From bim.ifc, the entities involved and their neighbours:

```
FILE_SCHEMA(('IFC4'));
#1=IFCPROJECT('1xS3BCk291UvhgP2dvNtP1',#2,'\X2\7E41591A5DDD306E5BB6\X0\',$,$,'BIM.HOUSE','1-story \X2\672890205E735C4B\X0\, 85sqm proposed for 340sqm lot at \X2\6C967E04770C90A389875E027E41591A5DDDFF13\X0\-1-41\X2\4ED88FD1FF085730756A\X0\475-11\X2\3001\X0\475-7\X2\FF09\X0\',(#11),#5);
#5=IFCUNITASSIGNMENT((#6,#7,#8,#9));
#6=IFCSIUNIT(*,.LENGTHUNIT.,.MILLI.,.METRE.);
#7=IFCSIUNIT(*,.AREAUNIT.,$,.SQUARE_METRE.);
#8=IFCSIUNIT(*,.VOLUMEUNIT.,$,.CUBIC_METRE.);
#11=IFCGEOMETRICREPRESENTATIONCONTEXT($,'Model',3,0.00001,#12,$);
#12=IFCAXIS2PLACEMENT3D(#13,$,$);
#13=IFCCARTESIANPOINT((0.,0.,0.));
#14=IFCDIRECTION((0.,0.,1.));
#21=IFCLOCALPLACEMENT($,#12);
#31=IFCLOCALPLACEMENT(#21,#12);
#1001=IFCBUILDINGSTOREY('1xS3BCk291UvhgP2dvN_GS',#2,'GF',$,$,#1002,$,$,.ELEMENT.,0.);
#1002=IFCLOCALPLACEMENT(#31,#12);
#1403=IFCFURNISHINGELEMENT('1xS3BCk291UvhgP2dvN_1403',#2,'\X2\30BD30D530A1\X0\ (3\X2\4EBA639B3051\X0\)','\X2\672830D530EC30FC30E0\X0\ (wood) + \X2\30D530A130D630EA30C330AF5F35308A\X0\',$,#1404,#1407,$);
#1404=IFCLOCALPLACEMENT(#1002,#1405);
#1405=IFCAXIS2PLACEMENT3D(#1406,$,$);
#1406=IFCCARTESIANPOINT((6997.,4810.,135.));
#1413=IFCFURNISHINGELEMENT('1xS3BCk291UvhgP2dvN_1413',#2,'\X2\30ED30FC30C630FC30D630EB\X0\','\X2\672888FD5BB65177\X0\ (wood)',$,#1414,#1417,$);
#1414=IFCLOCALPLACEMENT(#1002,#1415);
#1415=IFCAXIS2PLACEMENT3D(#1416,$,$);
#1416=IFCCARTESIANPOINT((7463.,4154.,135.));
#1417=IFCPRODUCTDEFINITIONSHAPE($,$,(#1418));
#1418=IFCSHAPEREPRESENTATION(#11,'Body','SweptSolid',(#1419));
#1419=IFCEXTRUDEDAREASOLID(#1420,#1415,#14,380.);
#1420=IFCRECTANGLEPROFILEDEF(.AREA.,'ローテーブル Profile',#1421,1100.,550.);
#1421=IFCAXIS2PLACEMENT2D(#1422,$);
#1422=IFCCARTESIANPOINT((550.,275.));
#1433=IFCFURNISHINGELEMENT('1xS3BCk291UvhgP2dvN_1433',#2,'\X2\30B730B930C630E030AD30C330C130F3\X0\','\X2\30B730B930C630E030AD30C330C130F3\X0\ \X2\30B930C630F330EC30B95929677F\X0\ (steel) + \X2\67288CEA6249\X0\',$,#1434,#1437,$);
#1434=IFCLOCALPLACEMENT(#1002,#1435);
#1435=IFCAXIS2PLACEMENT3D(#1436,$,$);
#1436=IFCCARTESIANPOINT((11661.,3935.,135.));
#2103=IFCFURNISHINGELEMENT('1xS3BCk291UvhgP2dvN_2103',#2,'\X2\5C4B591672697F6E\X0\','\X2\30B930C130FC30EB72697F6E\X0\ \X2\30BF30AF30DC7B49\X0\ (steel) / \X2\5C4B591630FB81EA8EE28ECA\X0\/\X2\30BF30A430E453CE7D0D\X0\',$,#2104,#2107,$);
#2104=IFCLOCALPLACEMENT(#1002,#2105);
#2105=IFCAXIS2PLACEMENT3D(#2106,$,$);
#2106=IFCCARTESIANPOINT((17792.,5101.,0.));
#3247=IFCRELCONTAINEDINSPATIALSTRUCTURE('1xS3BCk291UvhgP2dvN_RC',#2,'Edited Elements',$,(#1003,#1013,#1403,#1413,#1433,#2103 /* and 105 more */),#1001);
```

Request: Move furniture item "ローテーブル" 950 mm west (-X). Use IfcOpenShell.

```python
import ifcopenshell
import ifcopenshell.api.geometry
import ifcopenshell.util.placement
import ifcopenshell.util.unit

model = ifcopenshell.open("bim.ifc")
unit_scale = ifcopenshell.util.unit.calculate_unit_scale(model)

item = model.by_id(1413)
matrix = ifcopenshell.util.placement.get_local_placement(item.ObjectPlacement)
matrix[0, 3] -= 0.95 / unit_scale
ifcopenshell.api.geometry.edit_object_placement(model, product=item, matrix=matrix, is_si=False)

print(ifcopenshell.util.placement.get_local_placement(item.ObjectPlacement).round(3) + 0.0)

model.write("bim_updated.ifc")
```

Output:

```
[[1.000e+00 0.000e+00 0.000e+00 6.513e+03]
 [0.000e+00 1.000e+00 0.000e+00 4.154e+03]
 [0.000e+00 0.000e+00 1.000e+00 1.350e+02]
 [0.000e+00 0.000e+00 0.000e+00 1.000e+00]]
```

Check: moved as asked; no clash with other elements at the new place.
